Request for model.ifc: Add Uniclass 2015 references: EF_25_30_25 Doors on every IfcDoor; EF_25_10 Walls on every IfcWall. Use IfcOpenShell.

First a look at what the model holds.

```python
import ifcopenshell

model = ifcopenshell.open("model.ifc")
print(model.schema)
print("classifications:", [c.Name for c in model.by_type("IfcClassification")])
for ifc_class in ("IfcDoor", "IfcRoof", "IfcStair", "IfcWall", "IfcWindow"):
    print(ifc_class, len(model.by_type(ifc_class)))
```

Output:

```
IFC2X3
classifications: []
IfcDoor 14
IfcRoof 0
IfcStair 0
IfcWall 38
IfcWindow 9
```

```python
import ifcopenshell
import ifcopenshell.api.classification

model = ifcopenshell.open("model.ifc")

# IFC2X3 requires Source and Edition and has no link from the project to the system.
system = model.create_entity("IfcClassification", Source="NBS", Edition="2015", Name="Uniclass 2015")

codes = {
    "IfcDoor": ("EF_25_30_25", "Doors"),
    "IfcWall": ("EF_25_10", "Walls"),
}
for ifc_class, (code, name) in codes.items():
    products = model.by_type(ifc_class)
    ifcopenshell.api.classification.add_reference(
        model, products=products, classification=system, identification=code, name=name
    )
    print(code, len(products))

model.write("model_edited.ifc")
```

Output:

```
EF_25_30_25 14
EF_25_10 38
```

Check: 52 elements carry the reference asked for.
